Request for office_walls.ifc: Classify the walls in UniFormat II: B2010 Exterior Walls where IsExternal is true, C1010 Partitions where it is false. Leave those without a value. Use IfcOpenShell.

First a look at what the model holds.

```python
import ifcopenshell
import ifcopenshell.util.element

model = ifcopenshell.open("office_walls.ifc")
print(model.schema)
print("classifications:", [c.Name for c in model.by_type("IfcClassification")])
values = [ifcopenshell.util.element.get_pset(e, "Pset_WallCommon", "IsExternal") for e in model.by_type("IfcWall")]
for value in (True, False, None):
    print("IsExternal", value, values.count(value))
```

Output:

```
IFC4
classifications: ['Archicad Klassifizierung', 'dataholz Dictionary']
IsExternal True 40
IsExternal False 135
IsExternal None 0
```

```python
import ifcopenshell
import ifcopenshell.api.classification
import ifcopenshell.util.element

model = ifcopenshell.open("office_walls.ifc")

system = ifcopenshell.api.classification.add_classification(model, classification="UniFormat II")

walls = model.by_type("IfcWall")
external = {e: ifcopenshell.util.element.get_pset(e, "Pset_WallCommon", "IsExternal") for e in walls}
for flag, code, name in ((True, "B2010", "Exterior Walls"), (False, "C1010", "Partitions")):
    products = [e for e in walls if external[e] is flag]
    ifcopenshell.api.classification.add_reference(
        model, products=products, classification=system, identification=code, name=name
    )
    print(code, len(products))

model.write("office_walls-out.ifc")
```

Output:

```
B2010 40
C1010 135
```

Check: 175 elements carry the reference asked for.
